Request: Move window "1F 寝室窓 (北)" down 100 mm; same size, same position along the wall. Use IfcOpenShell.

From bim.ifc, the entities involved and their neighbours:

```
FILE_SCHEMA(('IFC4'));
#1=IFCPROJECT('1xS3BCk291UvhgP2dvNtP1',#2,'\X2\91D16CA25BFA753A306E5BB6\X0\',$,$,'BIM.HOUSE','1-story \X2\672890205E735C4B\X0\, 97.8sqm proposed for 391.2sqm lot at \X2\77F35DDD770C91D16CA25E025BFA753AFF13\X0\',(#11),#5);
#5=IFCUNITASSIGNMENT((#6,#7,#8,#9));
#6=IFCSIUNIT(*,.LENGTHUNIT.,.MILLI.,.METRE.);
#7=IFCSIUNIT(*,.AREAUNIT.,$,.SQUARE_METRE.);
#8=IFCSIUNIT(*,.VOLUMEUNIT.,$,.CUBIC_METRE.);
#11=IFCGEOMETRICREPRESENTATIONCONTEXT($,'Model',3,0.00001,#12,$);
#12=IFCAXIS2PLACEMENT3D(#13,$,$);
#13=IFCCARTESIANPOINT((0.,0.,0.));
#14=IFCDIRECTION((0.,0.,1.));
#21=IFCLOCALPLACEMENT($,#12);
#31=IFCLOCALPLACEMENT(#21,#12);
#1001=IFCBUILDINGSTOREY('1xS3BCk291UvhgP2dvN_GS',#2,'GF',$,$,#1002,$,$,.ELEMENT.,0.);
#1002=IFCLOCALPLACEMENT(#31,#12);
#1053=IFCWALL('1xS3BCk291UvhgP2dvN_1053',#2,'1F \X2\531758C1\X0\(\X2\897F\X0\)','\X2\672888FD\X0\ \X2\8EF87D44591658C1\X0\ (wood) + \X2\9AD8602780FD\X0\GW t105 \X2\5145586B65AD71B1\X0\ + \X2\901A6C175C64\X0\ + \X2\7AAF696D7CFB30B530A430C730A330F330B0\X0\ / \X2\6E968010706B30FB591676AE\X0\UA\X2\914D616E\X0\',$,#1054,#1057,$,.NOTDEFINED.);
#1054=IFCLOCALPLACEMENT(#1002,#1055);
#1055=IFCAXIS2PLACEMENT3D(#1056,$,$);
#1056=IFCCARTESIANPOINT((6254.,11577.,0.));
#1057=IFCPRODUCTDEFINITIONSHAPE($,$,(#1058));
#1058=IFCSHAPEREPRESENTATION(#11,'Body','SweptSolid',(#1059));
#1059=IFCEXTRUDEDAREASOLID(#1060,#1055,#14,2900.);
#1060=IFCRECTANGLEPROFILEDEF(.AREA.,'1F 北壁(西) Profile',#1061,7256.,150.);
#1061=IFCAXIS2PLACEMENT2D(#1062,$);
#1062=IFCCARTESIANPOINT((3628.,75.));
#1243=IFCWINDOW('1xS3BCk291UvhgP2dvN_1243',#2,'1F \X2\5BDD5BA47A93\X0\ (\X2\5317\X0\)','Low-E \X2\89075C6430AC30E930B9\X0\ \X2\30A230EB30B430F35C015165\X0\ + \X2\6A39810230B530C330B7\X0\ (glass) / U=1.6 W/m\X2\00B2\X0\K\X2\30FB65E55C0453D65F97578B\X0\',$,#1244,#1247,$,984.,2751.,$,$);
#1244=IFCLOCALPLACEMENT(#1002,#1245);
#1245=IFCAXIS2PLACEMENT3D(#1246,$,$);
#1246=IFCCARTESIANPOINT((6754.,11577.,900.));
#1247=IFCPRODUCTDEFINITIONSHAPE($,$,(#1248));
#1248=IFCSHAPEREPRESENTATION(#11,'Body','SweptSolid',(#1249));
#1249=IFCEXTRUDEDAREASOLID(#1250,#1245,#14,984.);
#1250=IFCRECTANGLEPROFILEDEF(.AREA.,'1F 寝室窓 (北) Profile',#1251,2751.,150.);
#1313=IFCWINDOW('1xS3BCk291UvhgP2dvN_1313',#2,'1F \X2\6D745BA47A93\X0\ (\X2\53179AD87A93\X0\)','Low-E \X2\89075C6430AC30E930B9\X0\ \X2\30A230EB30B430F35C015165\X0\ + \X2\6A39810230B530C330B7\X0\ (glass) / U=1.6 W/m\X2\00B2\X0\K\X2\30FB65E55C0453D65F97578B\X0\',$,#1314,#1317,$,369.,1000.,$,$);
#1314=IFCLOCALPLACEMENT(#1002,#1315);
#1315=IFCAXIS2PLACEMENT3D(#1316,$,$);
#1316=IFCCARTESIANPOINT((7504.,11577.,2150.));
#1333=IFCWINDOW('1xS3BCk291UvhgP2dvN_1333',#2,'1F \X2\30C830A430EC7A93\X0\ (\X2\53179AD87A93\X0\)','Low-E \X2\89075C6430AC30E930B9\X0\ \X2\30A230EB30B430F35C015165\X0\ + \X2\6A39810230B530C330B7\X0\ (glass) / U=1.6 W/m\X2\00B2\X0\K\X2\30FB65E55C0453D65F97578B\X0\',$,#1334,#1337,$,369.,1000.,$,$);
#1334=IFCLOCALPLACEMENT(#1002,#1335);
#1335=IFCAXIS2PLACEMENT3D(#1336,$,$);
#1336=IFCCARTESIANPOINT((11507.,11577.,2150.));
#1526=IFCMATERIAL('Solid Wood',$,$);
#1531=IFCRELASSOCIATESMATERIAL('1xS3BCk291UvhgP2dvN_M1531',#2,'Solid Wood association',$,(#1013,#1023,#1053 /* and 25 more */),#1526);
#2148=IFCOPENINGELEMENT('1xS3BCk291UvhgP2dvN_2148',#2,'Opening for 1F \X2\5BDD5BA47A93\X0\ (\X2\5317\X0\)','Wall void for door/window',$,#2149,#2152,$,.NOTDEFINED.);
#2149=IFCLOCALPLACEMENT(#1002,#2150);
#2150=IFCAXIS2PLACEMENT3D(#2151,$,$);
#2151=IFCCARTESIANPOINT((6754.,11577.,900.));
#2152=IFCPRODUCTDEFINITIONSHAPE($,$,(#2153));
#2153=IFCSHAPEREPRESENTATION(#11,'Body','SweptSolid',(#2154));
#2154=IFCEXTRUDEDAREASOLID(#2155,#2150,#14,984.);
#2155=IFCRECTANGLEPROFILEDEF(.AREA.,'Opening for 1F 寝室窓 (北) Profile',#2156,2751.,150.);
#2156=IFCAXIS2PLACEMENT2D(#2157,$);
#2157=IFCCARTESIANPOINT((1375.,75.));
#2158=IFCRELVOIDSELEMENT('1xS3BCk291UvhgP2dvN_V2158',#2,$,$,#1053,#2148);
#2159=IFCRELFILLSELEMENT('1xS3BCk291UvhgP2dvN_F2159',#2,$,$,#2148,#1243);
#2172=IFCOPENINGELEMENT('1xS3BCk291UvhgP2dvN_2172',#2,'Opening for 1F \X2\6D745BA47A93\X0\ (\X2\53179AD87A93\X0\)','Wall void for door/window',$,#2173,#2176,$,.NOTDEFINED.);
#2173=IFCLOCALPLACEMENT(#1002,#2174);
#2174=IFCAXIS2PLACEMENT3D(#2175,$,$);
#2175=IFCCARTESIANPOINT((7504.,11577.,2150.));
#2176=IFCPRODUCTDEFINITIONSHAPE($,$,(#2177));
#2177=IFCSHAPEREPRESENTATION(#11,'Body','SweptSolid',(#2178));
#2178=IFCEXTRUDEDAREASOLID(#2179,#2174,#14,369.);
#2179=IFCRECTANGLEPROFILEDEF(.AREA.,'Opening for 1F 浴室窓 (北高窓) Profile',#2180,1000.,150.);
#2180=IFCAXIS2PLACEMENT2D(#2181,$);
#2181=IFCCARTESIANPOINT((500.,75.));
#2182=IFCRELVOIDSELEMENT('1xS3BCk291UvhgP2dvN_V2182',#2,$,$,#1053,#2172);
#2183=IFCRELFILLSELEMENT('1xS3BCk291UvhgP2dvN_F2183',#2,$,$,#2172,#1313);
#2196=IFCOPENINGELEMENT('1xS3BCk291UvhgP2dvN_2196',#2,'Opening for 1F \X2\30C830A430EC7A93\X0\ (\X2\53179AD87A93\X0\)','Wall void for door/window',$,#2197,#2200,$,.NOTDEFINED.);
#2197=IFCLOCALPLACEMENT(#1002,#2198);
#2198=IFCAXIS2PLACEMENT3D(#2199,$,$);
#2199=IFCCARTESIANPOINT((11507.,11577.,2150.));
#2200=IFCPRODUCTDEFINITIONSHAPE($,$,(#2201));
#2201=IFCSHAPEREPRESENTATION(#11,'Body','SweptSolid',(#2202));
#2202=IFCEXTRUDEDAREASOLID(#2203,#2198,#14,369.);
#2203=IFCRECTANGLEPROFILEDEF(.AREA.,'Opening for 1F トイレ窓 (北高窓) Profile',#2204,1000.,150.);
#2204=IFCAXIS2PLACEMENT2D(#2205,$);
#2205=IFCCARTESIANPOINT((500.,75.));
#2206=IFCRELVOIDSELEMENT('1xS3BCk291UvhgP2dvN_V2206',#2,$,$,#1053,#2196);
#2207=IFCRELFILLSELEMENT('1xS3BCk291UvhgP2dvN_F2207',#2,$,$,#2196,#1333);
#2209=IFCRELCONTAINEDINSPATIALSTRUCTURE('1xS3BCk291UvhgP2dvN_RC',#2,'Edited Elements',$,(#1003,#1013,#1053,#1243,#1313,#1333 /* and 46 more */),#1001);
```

```python
import numpy as np
import ifcopenshell
import ifcopenshell.api.geometry
import ifcopenshell.util.placement
import ifcopenshell.util.unit

model = ifcopenshell.open("bim.ifc")
unit_scale = ifcopenshell.util.unit.calculate_unit_scale(model)

window = model.by_guid("1xS3BCk291UvhgP2dvN_1243")
opening = window.FillsVoids[0].RelatingOpeningElement
dz = -100.0

shift = np.array([0.0, 0.0, dz])
# The window is not placed relative to its opening, so move both.
for product in (opening, window):
    matrix = ifcopenshell.util.placement.get_local_placement(product.ObjectPlacement)
    matrix[:3, 3] += shift
    ifcopenshell.api.geometry.edit_object_placement(model, product=product, matrix=matrix, is_si=False)

print(f"moved by {dz * unit_scale:+.3f} m")

model.write("bim_rev.ifc")
```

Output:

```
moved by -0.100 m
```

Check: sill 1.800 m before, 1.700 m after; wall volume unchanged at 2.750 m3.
